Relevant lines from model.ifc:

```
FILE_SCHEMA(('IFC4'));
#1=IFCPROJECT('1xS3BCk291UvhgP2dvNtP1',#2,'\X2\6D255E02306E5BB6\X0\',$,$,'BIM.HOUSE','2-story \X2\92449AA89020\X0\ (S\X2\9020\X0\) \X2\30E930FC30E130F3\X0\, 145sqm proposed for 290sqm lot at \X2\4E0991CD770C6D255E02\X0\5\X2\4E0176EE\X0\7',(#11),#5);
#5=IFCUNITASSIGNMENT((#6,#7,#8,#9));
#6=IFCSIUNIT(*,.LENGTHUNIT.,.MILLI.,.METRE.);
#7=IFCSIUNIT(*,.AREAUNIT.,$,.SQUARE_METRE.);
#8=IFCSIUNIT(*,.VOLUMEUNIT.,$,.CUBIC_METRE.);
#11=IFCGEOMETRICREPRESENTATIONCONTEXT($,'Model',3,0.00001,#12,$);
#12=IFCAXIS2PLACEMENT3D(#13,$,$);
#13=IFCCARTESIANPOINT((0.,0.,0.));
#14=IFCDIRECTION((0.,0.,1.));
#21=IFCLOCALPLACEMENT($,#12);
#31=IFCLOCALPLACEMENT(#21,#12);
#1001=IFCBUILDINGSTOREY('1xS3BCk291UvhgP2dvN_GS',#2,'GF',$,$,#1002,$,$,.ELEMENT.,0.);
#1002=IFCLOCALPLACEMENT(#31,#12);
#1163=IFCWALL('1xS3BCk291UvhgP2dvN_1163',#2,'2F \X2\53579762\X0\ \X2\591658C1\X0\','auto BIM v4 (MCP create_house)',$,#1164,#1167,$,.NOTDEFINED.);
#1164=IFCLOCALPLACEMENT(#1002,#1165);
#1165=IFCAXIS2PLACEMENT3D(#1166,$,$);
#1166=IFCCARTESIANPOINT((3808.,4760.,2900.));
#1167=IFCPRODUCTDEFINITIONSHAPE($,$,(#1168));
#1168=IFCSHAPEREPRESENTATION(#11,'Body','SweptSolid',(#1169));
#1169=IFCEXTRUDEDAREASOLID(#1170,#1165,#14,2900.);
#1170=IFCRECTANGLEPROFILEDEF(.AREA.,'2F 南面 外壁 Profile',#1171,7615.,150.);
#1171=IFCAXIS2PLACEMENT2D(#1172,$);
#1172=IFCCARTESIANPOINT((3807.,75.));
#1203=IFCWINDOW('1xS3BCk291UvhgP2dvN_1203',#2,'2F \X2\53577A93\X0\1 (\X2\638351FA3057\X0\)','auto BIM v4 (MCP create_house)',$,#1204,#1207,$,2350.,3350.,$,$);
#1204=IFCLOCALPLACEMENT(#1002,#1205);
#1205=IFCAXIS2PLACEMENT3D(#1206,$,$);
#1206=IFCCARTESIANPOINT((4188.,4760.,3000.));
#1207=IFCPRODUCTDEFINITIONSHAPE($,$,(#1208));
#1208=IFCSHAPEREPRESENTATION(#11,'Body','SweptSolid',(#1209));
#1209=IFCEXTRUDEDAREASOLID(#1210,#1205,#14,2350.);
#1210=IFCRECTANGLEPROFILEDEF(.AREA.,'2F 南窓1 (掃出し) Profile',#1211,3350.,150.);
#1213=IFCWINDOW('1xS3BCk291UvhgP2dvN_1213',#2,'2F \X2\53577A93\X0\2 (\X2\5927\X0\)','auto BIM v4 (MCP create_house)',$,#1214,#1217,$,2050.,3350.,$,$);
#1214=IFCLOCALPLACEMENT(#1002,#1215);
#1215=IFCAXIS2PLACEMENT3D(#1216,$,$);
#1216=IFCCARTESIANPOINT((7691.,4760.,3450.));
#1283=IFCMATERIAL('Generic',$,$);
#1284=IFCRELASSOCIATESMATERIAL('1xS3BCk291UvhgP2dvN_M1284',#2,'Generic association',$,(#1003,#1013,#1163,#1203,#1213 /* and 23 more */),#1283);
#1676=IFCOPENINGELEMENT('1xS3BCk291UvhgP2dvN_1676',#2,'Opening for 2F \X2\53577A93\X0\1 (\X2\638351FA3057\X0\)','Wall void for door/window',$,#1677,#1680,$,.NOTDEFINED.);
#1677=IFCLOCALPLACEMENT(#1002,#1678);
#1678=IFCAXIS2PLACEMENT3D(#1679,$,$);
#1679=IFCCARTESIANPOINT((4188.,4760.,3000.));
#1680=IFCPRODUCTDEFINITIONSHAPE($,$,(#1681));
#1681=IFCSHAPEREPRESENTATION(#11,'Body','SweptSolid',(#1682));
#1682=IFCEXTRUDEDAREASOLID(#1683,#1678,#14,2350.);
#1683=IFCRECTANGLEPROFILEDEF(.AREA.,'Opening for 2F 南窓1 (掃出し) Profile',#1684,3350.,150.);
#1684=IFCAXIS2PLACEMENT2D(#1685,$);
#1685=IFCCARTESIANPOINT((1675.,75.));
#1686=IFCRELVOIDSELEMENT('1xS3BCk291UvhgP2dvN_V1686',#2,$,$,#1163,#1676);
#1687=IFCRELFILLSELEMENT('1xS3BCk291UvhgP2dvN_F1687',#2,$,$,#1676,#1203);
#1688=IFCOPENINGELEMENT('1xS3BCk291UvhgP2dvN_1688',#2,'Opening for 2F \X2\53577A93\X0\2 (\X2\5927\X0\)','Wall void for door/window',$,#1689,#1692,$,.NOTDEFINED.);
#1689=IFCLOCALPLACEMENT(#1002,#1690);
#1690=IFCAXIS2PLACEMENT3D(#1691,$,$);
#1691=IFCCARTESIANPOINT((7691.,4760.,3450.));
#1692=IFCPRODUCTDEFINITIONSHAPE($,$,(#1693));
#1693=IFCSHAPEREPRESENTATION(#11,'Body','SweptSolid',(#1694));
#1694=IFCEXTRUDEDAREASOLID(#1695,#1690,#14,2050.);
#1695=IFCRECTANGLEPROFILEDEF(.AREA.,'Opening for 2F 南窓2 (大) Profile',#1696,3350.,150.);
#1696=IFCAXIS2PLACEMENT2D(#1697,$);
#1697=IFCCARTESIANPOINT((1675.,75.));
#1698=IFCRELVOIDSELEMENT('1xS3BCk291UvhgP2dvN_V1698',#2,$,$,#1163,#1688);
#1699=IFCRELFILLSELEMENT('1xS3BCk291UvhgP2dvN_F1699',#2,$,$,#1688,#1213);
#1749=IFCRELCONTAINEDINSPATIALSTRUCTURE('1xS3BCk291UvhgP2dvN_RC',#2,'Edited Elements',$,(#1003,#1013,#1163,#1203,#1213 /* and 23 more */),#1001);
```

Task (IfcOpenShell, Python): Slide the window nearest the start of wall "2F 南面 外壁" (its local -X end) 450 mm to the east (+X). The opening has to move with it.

```python
import ifcopenshell
import ifcopenshell.api.geometry
import ifcopenshell.util.placement

model = ifcopenshell.open("model.ifc")

window = model.by_guid("1xS3BCk291UvhgP2dvN_1203")
opening = window.FillsVoids[0].RelatingOpeningElement
wall = opening.VoidsElements[0].RelatingBuildingElement

wall_matrix = ifcopenshell.util.placement.get_local_placement(wall.ObjectPlacement)
shift = wall_matrix[:3, 0] * 450.0
before = ifcopenshell.util.placement.get_local_placement(window.ObjectPlacement)[:3, 3].copy()

# The window is not placed relative to its opening, so move both.
for product in (opening, window):
    matrix = ifcopenshell.util.placement.get_local_placement(product.ObjectPlacement)
    matrix[:3, 3] += shift
    ifcopenshell.api.geometry.edit_object_placement(model, product=product, matrix=matrix, is_si=False)

after = ifcopenshell.util.placement.get_local_placement(window.ObjectPlacement)[:3, 3]
print("window moved by", (after - before).round(3) + 0.0)

model.write("model_v2.ifc")
```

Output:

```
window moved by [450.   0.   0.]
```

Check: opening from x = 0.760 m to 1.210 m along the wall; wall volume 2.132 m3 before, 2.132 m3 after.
